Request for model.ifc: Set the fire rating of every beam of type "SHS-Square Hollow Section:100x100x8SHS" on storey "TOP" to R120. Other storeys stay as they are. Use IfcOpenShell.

First a look at what the model holds.

```python
import ifcopenshell
import ifcopenshell.util.element

model = ifcopenshell.open("model.ifc")
print(model.schema)
storey = next(s for s in model.by_type("IfcBuildingStorey") if s.Name == "TOP")
beams = [e for e in ifcopenshell.util.element.get_decomposition(storey) if e.is_a("IfcBeam")]
seen = {}
for e in beams:
    element_type = ifcopenshell.util.element.get_type(e)
    key = (element_type.Name if element_type != e and element_type else None, ifcopenshell.util.element.get_pset(e, "Pset_BeamCommon", "FireRating"))
    seen[key] = seen.get(key, 0) + 1
for (name, value), count in sorted(seen.items(), key=str):
    print(count, "x", name, "|", value)
```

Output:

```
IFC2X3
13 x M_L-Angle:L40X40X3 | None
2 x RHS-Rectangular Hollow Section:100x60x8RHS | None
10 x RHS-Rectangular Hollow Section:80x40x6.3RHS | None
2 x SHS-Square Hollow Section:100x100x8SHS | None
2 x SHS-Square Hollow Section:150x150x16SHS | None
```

```python
import ifcopenshell
import ifcopenshell.api.pset
import ifcopenshell.util.element

model = ifcopenshell.open("model.ifc")

storey = next(s for s in model.by_type("IfcBuildingStorey") if s.Name == "TOP")
beams = [e for e in ifcopenshell.util.element.get_decomposition(storey) if e.is_a("IfcBeam")]

count = 0
for e in beams:
    element_type = ifcopenshell.util.element.get_type(e)
    if element_type in (None, e) or element_type.Name != "SHS-Square Hollow Section:100x100x8SHS":
        continue
    # add_pset returns the element's existing set when there is one.
    pset = ifcopenshell.api.pset.add_pset(model, product=e, name="Pset_BeamCommon")
    ifcopenshell.api.pset.edit_pset(model, pset=pset, properties={"FireRating": "R120"})
    count += 1

print(count, "beams updated")

model.write("model_edited.ifc")
```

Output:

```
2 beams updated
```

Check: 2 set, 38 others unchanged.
